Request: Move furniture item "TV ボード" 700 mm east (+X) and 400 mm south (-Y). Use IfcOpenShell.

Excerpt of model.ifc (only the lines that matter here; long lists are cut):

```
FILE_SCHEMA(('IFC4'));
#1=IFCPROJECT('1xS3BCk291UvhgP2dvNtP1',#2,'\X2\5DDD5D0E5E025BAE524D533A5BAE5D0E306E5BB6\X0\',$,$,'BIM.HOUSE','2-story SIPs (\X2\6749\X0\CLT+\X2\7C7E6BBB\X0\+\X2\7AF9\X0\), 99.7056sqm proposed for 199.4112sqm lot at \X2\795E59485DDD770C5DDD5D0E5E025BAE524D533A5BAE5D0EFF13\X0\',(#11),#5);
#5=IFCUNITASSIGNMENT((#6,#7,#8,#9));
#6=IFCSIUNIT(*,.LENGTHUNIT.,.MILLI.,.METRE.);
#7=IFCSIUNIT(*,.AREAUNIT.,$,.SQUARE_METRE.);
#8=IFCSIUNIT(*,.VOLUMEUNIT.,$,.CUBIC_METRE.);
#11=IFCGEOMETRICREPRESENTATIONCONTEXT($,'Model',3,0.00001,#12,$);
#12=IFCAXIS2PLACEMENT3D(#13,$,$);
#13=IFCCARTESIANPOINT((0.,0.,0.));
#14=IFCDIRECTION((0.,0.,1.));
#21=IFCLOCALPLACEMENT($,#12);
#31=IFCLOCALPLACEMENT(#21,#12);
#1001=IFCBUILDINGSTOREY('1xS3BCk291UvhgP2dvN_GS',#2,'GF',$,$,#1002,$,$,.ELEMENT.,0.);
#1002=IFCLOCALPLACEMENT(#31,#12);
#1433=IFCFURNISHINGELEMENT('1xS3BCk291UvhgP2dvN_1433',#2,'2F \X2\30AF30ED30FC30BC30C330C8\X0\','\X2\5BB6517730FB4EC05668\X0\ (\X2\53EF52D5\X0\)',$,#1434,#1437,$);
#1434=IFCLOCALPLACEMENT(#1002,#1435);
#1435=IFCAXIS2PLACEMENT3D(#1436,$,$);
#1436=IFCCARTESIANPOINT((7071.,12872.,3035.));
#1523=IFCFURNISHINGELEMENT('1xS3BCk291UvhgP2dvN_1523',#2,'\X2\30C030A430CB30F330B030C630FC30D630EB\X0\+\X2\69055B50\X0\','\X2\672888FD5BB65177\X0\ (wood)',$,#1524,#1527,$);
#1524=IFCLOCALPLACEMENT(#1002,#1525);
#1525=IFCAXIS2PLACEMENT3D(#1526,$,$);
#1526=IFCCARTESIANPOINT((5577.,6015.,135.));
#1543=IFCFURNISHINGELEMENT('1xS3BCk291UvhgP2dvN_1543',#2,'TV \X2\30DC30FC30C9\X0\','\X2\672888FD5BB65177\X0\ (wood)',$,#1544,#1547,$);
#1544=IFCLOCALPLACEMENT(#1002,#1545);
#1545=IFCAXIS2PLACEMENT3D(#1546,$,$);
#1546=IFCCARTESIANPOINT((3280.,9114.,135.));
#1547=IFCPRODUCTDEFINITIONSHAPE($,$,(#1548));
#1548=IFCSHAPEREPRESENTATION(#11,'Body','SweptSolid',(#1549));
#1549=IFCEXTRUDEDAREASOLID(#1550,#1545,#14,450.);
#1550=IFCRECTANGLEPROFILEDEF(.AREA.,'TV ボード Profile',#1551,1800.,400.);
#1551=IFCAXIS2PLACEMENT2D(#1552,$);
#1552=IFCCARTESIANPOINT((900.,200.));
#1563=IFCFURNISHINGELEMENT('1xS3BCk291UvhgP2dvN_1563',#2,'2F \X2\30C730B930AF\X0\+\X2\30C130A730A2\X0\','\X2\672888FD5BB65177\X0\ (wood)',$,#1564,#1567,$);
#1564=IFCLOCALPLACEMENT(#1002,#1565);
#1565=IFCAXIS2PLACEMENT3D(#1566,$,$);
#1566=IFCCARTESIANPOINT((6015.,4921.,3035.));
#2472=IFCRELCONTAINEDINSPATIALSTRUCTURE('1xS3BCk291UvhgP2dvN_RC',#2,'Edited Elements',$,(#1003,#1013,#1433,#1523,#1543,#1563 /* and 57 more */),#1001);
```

```python
import ifcopenshell
import ifcopenshell.api.geometry
import ifcopenshell.util.placement

model = ifcopenshell.open("model.ifc")

item = model.by_guid("1xS3BCk291UvhgP2dvN_1543")
matrix = ifcopenshell.util.placement.get_local_placement(item.ObjectPlacement)
matrix[0, 3] += 700.0
matrix[1, 3] -= 400.0
ifcopenshell.api.geometry.edit_object_placement(model, product=item, matrix=matrix, is_si=False)

print(ifcopenshell.util.placement.get_local_placement(item.ObjectPlacement).round(3) + 0.0)

model.write("model_rev.ifc")
```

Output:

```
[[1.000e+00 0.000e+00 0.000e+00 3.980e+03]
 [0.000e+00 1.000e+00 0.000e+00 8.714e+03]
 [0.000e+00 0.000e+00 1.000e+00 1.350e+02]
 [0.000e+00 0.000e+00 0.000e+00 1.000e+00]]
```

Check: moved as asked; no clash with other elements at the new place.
